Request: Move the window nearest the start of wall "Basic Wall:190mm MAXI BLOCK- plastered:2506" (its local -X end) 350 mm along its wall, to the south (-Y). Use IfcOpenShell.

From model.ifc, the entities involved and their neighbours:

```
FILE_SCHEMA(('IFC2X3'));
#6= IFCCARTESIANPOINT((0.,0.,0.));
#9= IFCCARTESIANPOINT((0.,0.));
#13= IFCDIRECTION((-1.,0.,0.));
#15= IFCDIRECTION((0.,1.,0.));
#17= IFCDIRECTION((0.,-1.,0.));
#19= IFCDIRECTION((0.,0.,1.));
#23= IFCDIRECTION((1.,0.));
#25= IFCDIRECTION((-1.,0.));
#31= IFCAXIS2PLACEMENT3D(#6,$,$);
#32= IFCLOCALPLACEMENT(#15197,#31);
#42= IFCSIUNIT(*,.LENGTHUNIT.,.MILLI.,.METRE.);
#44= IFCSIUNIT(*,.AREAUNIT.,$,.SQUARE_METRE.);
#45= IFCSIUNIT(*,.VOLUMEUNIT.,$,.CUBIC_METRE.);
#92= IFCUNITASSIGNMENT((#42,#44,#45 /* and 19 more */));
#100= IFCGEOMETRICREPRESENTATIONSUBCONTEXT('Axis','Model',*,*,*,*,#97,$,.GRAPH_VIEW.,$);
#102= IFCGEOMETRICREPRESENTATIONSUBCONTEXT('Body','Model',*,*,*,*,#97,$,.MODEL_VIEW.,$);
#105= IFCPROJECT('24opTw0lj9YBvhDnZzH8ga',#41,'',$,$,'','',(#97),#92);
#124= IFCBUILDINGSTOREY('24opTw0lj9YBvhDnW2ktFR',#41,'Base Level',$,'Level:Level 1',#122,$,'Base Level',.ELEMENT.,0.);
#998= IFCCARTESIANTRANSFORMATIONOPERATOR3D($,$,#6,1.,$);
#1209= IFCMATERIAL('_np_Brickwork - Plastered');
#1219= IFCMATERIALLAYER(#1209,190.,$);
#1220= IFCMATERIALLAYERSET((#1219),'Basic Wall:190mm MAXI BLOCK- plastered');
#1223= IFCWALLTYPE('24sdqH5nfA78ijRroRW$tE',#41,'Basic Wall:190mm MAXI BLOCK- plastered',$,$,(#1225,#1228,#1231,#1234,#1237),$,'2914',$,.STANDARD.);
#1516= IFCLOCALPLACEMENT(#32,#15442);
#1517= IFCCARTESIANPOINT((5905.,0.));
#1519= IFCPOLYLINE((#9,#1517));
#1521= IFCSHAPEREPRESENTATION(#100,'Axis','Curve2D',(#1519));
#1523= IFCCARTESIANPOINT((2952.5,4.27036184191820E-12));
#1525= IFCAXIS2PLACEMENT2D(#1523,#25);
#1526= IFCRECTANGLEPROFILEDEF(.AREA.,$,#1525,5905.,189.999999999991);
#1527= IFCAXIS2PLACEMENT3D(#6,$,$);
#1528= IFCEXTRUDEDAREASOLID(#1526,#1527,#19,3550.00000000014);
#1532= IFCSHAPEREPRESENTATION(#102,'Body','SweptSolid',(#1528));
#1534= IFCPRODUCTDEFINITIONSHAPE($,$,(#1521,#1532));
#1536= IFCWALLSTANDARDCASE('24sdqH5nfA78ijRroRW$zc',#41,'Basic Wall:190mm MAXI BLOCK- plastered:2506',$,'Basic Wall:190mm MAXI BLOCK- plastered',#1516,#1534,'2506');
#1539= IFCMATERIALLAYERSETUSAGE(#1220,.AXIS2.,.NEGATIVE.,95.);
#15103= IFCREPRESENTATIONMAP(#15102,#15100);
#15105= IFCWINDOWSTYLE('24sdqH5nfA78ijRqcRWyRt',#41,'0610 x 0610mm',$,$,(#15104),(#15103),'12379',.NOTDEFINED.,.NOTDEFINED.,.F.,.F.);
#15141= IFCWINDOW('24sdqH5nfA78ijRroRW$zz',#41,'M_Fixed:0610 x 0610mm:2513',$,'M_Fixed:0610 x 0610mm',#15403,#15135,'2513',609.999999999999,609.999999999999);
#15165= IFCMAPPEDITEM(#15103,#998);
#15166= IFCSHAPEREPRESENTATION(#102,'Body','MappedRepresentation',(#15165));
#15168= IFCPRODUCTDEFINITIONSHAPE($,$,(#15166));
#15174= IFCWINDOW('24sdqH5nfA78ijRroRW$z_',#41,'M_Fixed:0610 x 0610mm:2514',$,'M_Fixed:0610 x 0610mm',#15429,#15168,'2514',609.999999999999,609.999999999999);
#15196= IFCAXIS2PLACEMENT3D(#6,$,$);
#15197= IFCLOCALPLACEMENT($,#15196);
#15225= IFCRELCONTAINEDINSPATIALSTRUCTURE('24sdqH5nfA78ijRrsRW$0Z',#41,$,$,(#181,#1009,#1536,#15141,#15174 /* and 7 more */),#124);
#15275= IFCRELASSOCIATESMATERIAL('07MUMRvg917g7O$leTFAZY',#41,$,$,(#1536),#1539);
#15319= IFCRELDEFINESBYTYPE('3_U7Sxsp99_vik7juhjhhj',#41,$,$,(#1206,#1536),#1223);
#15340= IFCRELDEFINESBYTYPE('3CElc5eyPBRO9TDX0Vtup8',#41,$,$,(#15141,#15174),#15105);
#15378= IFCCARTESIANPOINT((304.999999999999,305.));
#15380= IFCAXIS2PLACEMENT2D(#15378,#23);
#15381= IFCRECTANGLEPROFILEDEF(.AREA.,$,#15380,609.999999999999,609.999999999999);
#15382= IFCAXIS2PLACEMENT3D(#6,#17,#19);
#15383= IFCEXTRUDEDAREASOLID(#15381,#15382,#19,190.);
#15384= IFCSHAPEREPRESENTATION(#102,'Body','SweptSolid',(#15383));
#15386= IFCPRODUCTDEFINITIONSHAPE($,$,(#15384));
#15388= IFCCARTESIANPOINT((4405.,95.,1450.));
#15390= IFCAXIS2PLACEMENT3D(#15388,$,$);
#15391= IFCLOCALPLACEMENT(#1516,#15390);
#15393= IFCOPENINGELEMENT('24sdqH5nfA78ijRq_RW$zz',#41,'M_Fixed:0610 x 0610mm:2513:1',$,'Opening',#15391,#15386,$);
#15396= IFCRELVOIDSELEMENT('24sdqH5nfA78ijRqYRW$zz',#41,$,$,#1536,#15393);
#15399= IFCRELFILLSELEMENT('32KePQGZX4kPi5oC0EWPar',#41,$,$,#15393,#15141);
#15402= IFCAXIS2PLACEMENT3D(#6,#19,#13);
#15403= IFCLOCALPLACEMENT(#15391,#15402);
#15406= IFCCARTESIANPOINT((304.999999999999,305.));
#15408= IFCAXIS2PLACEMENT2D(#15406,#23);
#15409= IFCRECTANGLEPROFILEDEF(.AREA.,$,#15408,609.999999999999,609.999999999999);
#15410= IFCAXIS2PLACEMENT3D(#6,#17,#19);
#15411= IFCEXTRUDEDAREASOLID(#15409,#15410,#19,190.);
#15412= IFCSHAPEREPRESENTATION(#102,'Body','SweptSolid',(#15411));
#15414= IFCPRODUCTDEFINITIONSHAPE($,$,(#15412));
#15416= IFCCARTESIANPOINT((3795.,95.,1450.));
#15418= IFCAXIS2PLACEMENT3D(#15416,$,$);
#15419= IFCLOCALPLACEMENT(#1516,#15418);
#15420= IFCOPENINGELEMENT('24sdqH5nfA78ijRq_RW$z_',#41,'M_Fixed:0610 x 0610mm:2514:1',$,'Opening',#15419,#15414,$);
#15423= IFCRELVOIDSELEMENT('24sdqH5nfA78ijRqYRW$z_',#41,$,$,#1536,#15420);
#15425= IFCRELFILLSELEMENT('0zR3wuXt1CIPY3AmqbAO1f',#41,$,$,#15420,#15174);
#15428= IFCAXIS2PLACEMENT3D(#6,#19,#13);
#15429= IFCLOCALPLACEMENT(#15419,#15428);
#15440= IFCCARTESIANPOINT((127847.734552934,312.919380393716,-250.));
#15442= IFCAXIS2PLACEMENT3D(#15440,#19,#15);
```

```python
import ifcopenshell
import ifcopenshell.api.geometry
import ifcopenshell.util.placement
import ifcopenshell.util.unit

model = ifcopenshell.open("model.ifc")
unit_scale = ifcopenshell.util.unit.calculate_unit_scale(model)

window = model.by_guid("24sdqH5nfA78ijRroRW$z_")
opening = window.FillsVoids[0].RelatingOpeningElement
wall = opening.VoidsElements[0].RelatingBuildingElement

wall_matrix = ifcopenshell.util.placement.get_local_placement(wall.ObjectPlacement)
shift = wall_matrix[:3, 0] * -0.35 / unit_scale
before = ifcopenshell.util.placement.get_local_placement(window.ObjectPlacement)[:3, 3].copy()

# The window is placed relative to its opening, so it follows when the opening moves.
matrix = ifcopenshell.util.placement.get_local_placement(opening.ObjectPlacement)
matrix[:3, 3] += shift
ifcopenshell.api.geometry.edit_object_placement(
    model, product=opening, matrix=matrix, is_si=False, should_transform_children=True
)

after = ifcopenshell.util.placement.get_local_placement(window.ObjectPlacement)[:3, 3]
print("window moved by", (after - before).round(3) + 0.0)

model.write("model_edited.ifc")
```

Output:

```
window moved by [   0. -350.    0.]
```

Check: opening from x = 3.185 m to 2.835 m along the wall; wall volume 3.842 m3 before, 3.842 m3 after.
